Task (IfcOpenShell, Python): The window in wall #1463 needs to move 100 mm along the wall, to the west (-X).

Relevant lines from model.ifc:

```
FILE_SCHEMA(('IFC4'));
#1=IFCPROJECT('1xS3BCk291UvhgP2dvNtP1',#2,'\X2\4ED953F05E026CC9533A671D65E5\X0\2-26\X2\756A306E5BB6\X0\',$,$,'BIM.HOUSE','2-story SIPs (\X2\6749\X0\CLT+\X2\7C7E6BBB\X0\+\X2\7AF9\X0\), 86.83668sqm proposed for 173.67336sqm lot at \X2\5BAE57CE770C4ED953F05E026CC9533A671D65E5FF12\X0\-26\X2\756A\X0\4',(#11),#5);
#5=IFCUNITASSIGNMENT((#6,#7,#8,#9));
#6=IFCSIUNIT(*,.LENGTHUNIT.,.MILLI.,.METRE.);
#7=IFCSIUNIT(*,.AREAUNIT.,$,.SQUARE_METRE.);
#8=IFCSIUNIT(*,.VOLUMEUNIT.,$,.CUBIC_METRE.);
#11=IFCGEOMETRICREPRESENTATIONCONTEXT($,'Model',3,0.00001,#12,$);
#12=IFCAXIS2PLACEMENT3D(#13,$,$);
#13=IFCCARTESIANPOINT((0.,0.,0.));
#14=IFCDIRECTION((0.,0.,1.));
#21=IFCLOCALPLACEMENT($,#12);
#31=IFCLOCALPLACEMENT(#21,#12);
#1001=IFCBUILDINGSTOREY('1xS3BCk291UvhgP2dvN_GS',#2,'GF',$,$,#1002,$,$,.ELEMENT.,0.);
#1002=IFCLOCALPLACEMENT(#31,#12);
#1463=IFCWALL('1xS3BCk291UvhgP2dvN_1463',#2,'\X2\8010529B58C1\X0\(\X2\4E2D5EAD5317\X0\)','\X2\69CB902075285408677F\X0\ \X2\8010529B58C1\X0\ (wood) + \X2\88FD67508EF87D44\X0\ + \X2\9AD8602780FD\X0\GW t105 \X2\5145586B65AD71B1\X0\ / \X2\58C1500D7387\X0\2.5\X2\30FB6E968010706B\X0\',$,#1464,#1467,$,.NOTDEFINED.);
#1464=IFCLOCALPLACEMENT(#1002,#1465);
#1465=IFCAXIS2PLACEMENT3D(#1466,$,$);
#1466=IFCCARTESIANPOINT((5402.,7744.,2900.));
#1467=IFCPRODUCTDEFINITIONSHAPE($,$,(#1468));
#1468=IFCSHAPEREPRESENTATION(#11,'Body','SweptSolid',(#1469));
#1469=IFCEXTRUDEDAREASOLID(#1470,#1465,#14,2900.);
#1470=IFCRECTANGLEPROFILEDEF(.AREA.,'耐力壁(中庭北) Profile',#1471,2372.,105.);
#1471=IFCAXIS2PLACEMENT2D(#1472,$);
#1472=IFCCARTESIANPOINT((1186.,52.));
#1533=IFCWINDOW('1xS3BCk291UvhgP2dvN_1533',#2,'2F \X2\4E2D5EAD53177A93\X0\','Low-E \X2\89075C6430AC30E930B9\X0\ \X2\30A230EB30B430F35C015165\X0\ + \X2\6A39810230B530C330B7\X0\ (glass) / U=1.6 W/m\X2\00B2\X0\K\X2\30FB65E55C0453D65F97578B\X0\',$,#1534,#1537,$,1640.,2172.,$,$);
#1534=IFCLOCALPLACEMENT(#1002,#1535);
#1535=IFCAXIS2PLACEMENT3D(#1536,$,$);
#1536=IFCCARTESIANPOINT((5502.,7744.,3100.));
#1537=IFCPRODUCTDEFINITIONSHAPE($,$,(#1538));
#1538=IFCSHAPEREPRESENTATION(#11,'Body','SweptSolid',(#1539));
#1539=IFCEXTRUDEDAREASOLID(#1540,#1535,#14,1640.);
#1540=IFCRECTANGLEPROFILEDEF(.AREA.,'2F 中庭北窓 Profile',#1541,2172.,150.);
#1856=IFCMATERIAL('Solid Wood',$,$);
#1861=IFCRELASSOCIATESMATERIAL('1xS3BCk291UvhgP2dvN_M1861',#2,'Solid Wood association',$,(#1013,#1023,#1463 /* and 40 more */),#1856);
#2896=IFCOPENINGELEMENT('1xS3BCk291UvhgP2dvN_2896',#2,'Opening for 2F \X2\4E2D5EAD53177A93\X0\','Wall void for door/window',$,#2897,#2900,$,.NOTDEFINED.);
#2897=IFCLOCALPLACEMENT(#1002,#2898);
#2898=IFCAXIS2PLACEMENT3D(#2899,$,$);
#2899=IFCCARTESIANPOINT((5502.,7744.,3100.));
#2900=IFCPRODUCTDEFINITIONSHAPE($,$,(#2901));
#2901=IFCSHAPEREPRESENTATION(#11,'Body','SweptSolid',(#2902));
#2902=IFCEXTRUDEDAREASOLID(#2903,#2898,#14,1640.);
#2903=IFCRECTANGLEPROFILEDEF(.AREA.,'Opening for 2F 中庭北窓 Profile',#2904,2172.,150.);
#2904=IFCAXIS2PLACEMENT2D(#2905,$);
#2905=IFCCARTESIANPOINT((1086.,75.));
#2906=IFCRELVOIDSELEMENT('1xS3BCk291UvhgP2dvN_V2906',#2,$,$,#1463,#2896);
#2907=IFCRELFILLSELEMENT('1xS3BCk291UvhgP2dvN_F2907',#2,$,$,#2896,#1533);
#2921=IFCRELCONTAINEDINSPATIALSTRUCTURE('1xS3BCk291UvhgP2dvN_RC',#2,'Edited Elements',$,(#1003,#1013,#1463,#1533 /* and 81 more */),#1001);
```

```python
import ifcopenshell
import ifcopenshell.api.geometry
import ifcopenshell.util.placement
import ifcopenshell.util.unit

model = ifcopenshell.open("model.ifc")
unit_scale = ifcopenshell.util.unit.calculate_unit_scale(model)

window = model.by_id(1533)
opening = window.FillsVoids[0].RelatingOpeningElement
wall = opening.VoidsElements[0].RelatingBuildingElement

wall_matrix = ifcopenshell.util.placement.get_local_placement(wall.ObjectPlacement)
shift = wall_matrix[:3, 0] * -0.1 / unit_scale
before = ifcopenshell.util.placement.get_local_placement(window.ObjectPlacement)[:3, 3].copy()

# The window is not placed relative to its opening, so move both.
for product in (opening, window):
    matrix = ifcopenshell.util.placement.get_local_placement(product.ObjectPlacement)
    matrix[:3, 3] += shift
    ifcopenshell.api.geometry.edit_object_placement(model, product=product, matrix=matrix, is_si=False)

after = ifcopenshell.util.placement.get_local_placement(window.ObjectPlacement)[:3, 3]
print("window moved by", (after - before).round(3) + 0.0)

model.write("model_v2.ifc")
```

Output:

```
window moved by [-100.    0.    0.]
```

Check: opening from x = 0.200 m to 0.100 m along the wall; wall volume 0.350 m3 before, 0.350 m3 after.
